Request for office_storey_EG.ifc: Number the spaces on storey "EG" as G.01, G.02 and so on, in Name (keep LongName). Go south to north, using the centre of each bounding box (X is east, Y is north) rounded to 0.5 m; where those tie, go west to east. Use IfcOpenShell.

First a look at what the model holds.

```python
import ifcopenshell
import ifcopenshell.util.element
import ifcopenshell.util.placement

model = ifcopenshell.open("office_storey_EG.ifc")
print(model.schema)
storey = next(s for s in model.by_type("IfcBuildingStorey") if s.Name == "EG")
spaces = [e for e in ifcopenshell.util.element.get_decomposition(storey) if e.is_a("IfcSpace")]
for e in sorted(spaces, key=lambda e: e.id()):
    origin = ifcopenshell.util.placement.get_local_placement(e.ObjectPlacement)[:3, 3]
    print(e.id(), e.Name, e.LongName, origin.round(2) + 0.0, sep=" | ")
```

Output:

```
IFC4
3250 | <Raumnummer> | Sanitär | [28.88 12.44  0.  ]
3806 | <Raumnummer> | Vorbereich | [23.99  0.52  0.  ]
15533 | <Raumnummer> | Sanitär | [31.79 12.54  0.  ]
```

```python
import ifcopenshell
import ifcopenshell.geom
import ifcopenshell.util.element
import ifcopenshell.util.shape

model = ifcopenshell.open("office_storey_EG.ifc")
settings = ifcopenshell.geom.settings()
settings.set("use-world-coords", True)


def centre(element):
    shape = ifcopenshell.geom.create_shape(settings, element)
    return ifcopenshell.util.shape.get_bbox_centroid(shape.geometry)


storey = next(s for s in model.by_type("IfcBuildingStorey") if s.Name == "EG")
spaces = [e for e in ifcopenshell.util.element.get_decomposition(storey) if e.is_a("IfcSpace")]

# Insertion points can sit at a corner or the storey origin, so sort by the geometry (in metres).
centres = {e: centre(e) for e in spaces}
spaces.sort(key=lambda e: (round(centres[e][1] / 0.5), centres[e][0]))

for i, e in enumerate(spaces, start=1):
    number = f"G.{i:02d}"
    e.Name = number
    print(e.id(), number)

model.write("office_storey_EG-out.ifc")
```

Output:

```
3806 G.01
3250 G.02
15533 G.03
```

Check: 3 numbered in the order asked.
